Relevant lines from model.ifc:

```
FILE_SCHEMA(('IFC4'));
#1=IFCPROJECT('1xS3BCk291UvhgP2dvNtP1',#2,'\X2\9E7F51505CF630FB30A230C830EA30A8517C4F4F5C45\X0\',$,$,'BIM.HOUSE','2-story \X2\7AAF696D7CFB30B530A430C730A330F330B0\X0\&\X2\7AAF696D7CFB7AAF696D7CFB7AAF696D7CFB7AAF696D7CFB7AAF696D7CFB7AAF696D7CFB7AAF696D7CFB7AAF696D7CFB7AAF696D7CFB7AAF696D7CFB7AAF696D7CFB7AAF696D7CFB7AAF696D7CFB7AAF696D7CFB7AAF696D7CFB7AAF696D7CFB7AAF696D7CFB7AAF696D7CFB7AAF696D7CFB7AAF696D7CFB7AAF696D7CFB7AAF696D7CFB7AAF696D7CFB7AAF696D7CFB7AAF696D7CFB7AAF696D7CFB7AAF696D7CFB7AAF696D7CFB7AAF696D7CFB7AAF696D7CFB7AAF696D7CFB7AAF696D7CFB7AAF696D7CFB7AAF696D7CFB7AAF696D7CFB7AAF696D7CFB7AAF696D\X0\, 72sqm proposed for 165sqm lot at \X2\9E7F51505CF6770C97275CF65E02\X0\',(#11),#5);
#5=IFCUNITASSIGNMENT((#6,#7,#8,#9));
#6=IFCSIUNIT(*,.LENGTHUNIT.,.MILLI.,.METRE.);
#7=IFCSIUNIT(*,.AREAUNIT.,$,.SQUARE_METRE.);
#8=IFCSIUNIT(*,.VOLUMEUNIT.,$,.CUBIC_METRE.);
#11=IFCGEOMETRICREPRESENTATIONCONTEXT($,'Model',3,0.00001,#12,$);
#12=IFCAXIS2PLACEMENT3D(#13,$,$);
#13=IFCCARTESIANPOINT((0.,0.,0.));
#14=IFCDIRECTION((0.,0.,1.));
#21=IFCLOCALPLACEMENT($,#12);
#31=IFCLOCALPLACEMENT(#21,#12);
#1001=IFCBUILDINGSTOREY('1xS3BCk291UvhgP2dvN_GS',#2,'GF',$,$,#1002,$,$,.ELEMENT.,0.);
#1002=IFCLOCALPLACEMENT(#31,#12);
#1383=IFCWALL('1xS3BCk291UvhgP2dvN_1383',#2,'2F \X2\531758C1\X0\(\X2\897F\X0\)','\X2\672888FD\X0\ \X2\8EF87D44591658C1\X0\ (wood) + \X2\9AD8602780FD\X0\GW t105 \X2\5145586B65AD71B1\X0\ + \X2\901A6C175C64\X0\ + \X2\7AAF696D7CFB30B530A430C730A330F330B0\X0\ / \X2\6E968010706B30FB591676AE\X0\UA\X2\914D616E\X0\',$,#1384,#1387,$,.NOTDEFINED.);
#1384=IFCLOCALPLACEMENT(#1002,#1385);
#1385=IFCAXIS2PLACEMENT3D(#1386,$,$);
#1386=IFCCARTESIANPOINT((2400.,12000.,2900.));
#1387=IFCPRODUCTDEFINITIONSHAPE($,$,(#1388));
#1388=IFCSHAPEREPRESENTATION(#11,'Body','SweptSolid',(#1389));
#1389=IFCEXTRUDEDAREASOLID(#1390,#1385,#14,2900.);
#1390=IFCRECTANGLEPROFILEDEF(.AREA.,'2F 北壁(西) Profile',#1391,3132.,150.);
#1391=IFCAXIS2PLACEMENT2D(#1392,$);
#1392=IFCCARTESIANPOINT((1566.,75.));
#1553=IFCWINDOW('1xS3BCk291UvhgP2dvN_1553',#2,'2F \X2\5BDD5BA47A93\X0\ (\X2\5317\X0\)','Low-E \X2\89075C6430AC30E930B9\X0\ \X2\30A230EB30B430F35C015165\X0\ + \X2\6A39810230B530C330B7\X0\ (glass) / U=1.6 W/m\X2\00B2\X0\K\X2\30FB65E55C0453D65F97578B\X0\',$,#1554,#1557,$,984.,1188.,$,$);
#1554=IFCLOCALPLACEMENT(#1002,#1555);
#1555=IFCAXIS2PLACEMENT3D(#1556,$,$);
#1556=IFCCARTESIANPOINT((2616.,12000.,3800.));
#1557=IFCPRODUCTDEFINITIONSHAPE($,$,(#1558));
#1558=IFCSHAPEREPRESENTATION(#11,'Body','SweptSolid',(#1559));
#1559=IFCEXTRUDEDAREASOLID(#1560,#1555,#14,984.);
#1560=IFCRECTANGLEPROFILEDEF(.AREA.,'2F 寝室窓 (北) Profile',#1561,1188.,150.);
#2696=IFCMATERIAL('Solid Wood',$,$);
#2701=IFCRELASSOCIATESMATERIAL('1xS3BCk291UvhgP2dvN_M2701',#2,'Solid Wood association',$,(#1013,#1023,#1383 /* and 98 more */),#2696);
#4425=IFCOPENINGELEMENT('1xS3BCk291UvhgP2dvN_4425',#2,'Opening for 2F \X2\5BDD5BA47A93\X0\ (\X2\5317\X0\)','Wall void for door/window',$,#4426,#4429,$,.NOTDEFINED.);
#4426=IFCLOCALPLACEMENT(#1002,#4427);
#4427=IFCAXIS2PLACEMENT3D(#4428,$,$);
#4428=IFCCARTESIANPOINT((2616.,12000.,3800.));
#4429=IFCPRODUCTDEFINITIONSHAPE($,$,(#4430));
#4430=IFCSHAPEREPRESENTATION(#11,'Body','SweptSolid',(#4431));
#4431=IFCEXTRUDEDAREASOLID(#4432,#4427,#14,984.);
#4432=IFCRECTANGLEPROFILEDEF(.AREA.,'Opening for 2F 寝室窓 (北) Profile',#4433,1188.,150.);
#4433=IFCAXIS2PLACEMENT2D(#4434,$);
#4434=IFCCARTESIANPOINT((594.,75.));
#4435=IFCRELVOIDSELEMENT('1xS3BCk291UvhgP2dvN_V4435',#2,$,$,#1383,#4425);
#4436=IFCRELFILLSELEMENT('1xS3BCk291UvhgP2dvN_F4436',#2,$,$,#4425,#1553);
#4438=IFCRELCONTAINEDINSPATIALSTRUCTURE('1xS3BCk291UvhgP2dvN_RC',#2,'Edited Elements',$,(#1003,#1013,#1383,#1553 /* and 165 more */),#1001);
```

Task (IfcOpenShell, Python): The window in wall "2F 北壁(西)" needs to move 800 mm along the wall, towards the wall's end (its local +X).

```python
import ifcopenshell
import ifcopenshell.api.geometry
import ifcopenshell.util.placement
import ifcopenshell.util.unit

model = ifcopenshell.open("model.ifc")
unit_scale = ifcopenshell.util.unit.calculate_unit_scale(model)

window = model.by_guid("1xS3BCk291UvhgP2dvN_1553")
opening = window.FillsVoids[0].RelatingOpeningElement
wall = opening.VoidsElements[0].RelatingBuildingElement

wall_matrix = ifcopenshell.util.placement.get_local_placement(wall.ObjectPlacement)
shift = wall_matrix[:3, 0] * 0.8 / unit_scale
before = ifcopenshell.util.placement.get_local_placement(window.ObjectPlacement)[:3, 3].copy()

# The window is not placed relative to its opening, so move both.
for product in (opening, window):
    matrix = ifcopenshell.util.placement.get_local_placement(product.ObjectPlacement)
    matrix[:3, 3] += shift
    ifcopenshell.api.geometry.edit_object_placement(model, product=product, matrix=matrix, is_si=False)

after = ifcopenshell.util.placement.get_local_placement(window.ObjectPlacement)[:3, 3]
print("window moved by", (after - before).round(3) + 0.0)

model.write("model-out.ifc")
```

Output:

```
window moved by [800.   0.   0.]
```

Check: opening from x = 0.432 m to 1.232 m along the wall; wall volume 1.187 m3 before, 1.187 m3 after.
